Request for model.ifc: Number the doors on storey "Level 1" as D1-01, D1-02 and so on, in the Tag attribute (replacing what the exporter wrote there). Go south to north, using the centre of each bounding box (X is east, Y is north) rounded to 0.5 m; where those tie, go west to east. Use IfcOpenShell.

First a look at what the model holds.

```python
import ifcopenshell
import ifcopenshell.util.element
import ifcopenshell.util.placement

model = ifcopenshell.open("model.ifc")
print(model.schema)
storey = next(s for s in model.by_type("IfcBuildingStorey") if s.Name == "Level 1")
doors = [e for e in ifcopenshell.util.element.get_decomposition(storey) if e.is_a("IfcDoor")]
for e in sorted(doors, key=lambda e: e.id()):
    origin = ifcopenshell.util.placement.get_local_placement(e.ObjectPlacement)[:3, 3]
    print(e.id(), e.Tag, e.Name, origin.round(2) + 0.0, sep=" | ")
```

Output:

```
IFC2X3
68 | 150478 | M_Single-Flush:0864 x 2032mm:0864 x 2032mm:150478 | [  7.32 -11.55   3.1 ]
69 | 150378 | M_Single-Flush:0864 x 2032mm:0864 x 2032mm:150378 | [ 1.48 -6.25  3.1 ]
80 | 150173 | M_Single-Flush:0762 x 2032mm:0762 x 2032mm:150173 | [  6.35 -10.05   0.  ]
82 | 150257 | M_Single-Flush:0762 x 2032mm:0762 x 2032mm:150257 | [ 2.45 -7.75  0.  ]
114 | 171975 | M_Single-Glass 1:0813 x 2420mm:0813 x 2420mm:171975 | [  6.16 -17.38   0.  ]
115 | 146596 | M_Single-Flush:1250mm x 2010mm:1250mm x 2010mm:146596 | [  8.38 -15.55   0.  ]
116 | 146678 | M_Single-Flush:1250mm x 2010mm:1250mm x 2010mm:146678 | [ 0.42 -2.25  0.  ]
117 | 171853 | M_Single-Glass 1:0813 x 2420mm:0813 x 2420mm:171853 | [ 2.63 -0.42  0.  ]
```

```python
import ifcopenshell
import ifcopenshell.geom
import ifcopenshell.util.element
import ifcopenshell.util.shape

model = ifcopenshell.open("model.ifc")
settings = ifcopenshell.geom.settings()
settings.set("use-world-coords", True)


def centre(element):
    shape = ifcopenshell.geom.create_shape(settings, element)
    return ifcopenshell.util.shape.get_bbox_centroid(shape.geometry)


storey = next(s for s in model.by_type("IfcBuildingStorey") if s.Name == "Level 1")
doors = [e for e in ifcopenshell.util.element.get_decomposition(storey) if e.is_a("IfcDoor")]

# Insertion points can sit at a corner or the storey origin, so sort by the geometry (in metres).
centres = {e: centre(e) for e in doors}
doors.sort(key=lambda e: (round(centres[e][1] / 0.5), centres[e][0]))

for i, e in enumerate(doors, start=1):
    number = f"D1-{i:02d}"
    e.Tag = number
    print(e.id(), number)

model.write("model_edited.ifc")
```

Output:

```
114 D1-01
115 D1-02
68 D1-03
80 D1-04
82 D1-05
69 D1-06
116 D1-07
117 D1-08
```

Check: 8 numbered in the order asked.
